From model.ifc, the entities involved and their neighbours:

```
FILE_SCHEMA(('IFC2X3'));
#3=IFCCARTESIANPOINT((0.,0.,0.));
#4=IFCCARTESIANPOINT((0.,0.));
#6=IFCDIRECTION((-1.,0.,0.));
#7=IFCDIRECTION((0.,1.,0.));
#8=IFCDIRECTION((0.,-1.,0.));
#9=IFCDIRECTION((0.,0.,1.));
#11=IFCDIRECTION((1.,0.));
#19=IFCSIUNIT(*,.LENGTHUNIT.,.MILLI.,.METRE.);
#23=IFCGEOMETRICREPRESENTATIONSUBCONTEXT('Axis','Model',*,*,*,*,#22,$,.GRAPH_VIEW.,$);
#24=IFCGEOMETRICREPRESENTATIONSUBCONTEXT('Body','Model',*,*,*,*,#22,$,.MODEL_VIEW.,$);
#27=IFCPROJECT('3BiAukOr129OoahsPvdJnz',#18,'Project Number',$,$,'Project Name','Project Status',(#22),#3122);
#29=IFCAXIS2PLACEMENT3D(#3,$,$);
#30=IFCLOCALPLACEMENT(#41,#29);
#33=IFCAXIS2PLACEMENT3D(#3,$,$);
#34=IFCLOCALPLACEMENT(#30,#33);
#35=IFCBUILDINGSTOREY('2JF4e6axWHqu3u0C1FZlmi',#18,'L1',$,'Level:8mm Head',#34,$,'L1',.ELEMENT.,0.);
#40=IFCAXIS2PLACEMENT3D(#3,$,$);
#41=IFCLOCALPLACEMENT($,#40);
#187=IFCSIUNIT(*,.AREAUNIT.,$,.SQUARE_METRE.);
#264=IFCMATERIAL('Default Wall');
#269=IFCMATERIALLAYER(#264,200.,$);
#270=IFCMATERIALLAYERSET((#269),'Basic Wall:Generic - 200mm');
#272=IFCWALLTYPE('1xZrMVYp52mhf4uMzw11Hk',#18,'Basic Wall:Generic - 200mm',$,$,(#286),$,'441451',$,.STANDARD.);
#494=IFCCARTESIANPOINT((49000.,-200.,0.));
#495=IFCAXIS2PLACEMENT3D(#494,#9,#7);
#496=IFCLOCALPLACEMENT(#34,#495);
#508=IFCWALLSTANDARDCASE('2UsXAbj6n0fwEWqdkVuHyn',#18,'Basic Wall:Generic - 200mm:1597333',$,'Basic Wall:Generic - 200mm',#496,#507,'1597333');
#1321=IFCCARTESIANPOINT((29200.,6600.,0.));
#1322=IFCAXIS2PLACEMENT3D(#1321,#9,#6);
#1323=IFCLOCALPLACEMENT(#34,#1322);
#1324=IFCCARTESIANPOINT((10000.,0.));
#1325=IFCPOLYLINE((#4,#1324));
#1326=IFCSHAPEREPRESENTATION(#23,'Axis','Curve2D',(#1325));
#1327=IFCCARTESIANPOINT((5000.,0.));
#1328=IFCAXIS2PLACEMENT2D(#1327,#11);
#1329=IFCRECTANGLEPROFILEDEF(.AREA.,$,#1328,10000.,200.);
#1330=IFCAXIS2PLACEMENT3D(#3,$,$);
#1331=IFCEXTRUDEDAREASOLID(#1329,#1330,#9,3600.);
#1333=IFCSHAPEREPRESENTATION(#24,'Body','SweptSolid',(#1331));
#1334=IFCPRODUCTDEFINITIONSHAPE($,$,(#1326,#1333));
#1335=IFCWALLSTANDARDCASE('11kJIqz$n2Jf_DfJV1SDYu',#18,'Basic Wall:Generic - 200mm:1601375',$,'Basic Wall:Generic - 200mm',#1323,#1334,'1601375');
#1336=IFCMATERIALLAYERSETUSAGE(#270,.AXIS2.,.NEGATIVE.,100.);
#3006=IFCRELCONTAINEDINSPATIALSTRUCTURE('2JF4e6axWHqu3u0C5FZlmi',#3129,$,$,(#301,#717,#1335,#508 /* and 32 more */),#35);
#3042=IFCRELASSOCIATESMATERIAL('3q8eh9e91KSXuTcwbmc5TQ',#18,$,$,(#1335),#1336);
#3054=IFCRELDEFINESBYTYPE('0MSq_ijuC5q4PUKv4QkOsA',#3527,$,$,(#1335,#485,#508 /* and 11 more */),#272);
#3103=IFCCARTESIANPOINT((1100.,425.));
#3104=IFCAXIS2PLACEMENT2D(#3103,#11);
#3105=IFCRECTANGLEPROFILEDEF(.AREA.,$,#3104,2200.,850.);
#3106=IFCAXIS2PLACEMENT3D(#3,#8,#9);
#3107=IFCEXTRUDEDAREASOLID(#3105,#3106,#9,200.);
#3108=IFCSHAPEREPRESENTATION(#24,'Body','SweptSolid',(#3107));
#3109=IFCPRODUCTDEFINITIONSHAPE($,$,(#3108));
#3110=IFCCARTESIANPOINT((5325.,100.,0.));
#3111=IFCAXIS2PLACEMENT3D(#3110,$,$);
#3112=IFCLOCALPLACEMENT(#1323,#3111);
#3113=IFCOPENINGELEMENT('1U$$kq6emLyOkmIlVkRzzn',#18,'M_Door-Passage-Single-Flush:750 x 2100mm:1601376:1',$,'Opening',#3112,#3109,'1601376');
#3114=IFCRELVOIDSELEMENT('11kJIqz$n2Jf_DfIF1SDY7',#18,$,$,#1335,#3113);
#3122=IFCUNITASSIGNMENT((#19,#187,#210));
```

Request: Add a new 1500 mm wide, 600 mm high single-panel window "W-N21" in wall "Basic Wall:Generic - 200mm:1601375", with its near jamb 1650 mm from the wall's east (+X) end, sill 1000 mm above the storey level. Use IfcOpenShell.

```python
import numpy as np
import ifcopenshell
import ifcopenshell.api.feature
import ifcopenshell.api.geometry
import ifcopenshell.api.root
import ifcopenshell.api.spatial
import ifcopenshell.api.type
import ifcopenshell.geom
import ifcopenshell.util.element
import ifcopenshell.util.placement
import ifcopenshell.util.representation
import ifcopenshell.util.shape
import ifcopenshell.util.unit

model = ifcopenshell.open("model.ifc")
unit_scale = ifcopenshell.util.unit.calculate_unit_scale(model)
settings = ifcopenshell.geom.settings()


def volume(element):
    """Net volume in cubic metres, openings subtracted."""
    shape = ifcopenshell.geom.create_shape(settings, element)
    return ifcopenshell.util.shape.get_volume(shape.geometry)


wall = model.by_guid("11kJIqz$n2Jf_DfJV1SDYu")
storey = ifcopenshell.util.element.get_container(wall, ifc_class="IfcBuildingStorey")
context = ifcopenshell.util.representation.get_context(model, "Model", "Body", "MODEL_VIEW")
before = volume(wall)

width, height, from_end, sill = 1.5, 0.6, 1.65, 1  # metres

# The wall runs along its own X axis, and the end named is its -X end.
wall_shape = ifcopenshell.geom.create_shape(settings, wall)
x, y, z = ifcopenshell.util.shape.get_vertices(wall_shape.geometry).T
start = x.min() + from_end
face, thickness = float(y.min()), float(y.max() - y.min())
wall_matrix = ifcopenshell.util.placement.get_local_placement(wall.ObjectPlacement)
level = ifcopenshell.util.placement.get_local_placement(storey.ObjectPlacement)[2, 3]


def in_wall(x, y):
    """Placement at x, y metres in the wall's axes, at sill height."""
    matrix = wall_matrix.copy()
    matrix[:, 3] = wall_matrix @ np.array([x / unit_scale, y / unit_scale, 0.0, 1.0])
    matrix[2, 3] = level + sill / unit_scale
    return matrix


# Opening: a box that overshoots both wall faces by 50 mm.
opening = ifcopenshell.api.root.create_entity(model, ifc_class="IfcOpeningElement")
box = ifcopenshell.api.geometry.add_wall_representation(
    model, context=context, length=width, height=height, thickness=thickness + 0.1
)
ifcopenshell.api.geometry.assign_representation(model, product=opening, representation=box)
ifcopenshell.api.geometry.edit_object_placement(model, product=opening, matrix=in_wall(start, face - 0.05), is_si=False)
ifcopenshell.api.feature.add_feature(model, feature=opening, element=wall)

window = ifcopenshell.api.root.create_entity(model, ifc_class="IfcWindow", name="W-N21")
window.OverallWidth, window.OverallHeight = width / unit_scale, height / unit_scale
body = ifcopenshell.api.geometry.add_window_representation(
    model,
    context=context,
    overall_width=window.OverallWidth,
    overall_height=window.OverallHeight,
    partition_type="SINGLE_PANEL",
)
ifcopenshell.api.geometry.assign_representation(model, product=window, representation=body)
ifcopenshell.api.spatial.assign_container(model, products=[window], relating_structure=storey)
fills = ifcopenshell.api.feature.add_filling(model, opening=opening, element=window)
fills.OwnerHistory = window.OwnerHistory  # required in IFC2X3

# IFC2X3 keeps the operation on the window style.
style = ifcopenshell.api.root.create_entity(model, ifc_class="IfcWindowStyle", name="W-N21")
style.OperationType, style.ConstructionType = "SINGLE_PANEL", "NOTDEFINED"
style.ParameterTakesPrecedence = style.Sizeable = False
ifcopenshell.api.type.assign_type(model, related_objects=[window], relating_type=style)

# Centre the window in the wall's thickness.
ifcopenshell.api.geometry.edit_object_placement(model, product=window, matrix=in_wall(start, face), is_si=False)
window_shape = ifcopenshell.geom.create_shape(settings, window)
depth = ifcopenshell.util.shape.get_vertices(window_shape.geometry)[:, 1]
offset = face + thickness / 2 - (depth.min() + depth.max()) / 2
ifcopenshell.api.geometry.edit_object_placement(model, product=window, matrix=in_wall(start, offset), is_si=False)

after = volume(wall)

print(f"wall volume {before:.3f} -> {after:.3f} m3")

model.write("model_v2.ifc")
```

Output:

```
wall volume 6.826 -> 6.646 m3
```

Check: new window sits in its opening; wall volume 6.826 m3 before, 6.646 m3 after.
